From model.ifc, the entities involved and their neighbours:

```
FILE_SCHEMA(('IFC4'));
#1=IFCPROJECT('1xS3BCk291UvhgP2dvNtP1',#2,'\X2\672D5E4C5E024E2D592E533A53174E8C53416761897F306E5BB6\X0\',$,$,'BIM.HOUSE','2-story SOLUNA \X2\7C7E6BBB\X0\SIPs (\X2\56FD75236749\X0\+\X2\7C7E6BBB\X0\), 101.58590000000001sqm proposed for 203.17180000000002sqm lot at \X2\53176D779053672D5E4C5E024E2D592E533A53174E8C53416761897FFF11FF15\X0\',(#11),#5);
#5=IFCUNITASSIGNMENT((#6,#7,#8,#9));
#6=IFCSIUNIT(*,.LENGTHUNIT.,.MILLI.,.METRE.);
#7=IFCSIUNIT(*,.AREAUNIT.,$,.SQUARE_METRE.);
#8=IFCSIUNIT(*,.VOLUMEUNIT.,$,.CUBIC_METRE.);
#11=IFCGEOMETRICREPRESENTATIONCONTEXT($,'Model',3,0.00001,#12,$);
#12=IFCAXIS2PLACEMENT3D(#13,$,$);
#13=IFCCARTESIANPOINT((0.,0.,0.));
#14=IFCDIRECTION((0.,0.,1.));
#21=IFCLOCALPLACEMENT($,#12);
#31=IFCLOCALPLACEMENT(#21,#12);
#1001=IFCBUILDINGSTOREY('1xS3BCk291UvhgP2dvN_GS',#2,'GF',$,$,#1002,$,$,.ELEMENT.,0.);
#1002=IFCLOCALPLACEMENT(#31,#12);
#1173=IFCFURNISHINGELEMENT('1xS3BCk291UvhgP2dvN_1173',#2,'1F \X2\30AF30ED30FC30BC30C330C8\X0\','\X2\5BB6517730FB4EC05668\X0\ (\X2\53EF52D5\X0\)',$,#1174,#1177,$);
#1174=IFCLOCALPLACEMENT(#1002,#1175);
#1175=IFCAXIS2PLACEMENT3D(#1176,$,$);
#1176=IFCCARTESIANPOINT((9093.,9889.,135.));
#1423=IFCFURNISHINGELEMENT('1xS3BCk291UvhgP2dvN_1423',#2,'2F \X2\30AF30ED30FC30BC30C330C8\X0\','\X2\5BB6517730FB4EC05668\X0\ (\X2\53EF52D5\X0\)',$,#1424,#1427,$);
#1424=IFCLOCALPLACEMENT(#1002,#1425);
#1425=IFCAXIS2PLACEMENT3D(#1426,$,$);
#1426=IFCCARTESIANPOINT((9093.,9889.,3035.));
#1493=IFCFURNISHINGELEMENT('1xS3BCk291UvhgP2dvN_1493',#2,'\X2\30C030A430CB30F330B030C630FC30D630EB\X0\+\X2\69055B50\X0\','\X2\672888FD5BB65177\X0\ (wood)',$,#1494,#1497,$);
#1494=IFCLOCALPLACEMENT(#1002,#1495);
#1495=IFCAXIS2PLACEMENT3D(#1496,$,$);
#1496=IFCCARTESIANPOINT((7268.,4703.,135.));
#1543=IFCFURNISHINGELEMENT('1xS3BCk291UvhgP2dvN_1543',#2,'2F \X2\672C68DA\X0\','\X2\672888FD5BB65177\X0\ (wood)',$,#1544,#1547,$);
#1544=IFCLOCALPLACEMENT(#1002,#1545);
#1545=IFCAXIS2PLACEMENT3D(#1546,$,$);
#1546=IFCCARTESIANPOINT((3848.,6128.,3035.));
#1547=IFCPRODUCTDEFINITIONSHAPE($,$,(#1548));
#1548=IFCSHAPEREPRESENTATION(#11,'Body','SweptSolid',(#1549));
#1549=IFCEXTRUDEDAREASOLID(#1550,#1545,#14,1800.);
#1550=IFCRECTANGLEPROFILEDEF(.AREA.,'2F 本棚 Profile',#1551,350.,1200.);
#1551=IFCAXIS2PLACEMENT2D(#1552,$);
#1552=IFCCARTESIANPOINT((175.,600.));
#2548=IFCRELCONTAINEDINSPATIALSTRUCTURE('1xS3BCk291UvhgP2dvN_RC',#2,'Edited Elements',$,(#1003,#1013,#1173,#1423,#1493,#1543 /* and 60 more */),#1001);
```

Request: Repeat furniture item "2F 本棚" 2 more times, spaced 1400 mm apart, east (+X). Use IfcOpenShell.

```python
import numpy as np
import ifcopenshell
import ifcopenshell.api.geometry
import ifcopenshell.api.root
import ifcopenshell.util.element
import ifcopenshell.util.placement
import ifcopenshell.util.unit

model = ifcopenshell.open("model.ifc")
unit_scale = ifcopenshell.util.unit.calculate_unit_scale(model)


def reuse_history(source, copy):
    """copy_class also copies each property set's owner history, people and application; keep the originals."""
    for rel in copy.IsDefinedBy:
        if rel.is_a("IfcRelDefinesByProperties") and (history := rel.RelatingPropertyDefinition.OwnerHistory):
            rel.RelatingPropertyDefinition.OwnerHistory = source.OwnerHistory
            ifcopenshell.util.element.remove_deep2(model, history)


source = model.by_guid("1xS3BCk291UvhgP2dvN_1543")
base = ifcopenshell.util.placement.get_local_placement(source.ObjectPlacement)
step = np.array([1.0, 0.0, 0.0]) * 1.4 / unit_scale

for i in range(1, 3):
    copy = ifcopenshell.api.root.copy_class(model, product=source)
    copy.Representation = ifcopenshell.util.element.copy_deep(
        model, source.Representation, exclude=["IfcGeometricRepresentationContext", "IfcRepresentationMap"]
    )
    reuse_history(source, copy)
    matrix = base.copy()
    matrix[:3, 3] += i * step
    print("added at", matrix[:3, 3].round(3) + 0.0)
    ifcopenshell.api.geometry.edit_object_placement(model, product=copy, matrix=matrix, is_si=False)

model.write("model_edited.ifc")
```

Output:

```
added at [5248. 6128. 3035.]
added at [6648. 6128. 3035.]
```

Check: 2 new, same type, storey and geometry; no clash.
